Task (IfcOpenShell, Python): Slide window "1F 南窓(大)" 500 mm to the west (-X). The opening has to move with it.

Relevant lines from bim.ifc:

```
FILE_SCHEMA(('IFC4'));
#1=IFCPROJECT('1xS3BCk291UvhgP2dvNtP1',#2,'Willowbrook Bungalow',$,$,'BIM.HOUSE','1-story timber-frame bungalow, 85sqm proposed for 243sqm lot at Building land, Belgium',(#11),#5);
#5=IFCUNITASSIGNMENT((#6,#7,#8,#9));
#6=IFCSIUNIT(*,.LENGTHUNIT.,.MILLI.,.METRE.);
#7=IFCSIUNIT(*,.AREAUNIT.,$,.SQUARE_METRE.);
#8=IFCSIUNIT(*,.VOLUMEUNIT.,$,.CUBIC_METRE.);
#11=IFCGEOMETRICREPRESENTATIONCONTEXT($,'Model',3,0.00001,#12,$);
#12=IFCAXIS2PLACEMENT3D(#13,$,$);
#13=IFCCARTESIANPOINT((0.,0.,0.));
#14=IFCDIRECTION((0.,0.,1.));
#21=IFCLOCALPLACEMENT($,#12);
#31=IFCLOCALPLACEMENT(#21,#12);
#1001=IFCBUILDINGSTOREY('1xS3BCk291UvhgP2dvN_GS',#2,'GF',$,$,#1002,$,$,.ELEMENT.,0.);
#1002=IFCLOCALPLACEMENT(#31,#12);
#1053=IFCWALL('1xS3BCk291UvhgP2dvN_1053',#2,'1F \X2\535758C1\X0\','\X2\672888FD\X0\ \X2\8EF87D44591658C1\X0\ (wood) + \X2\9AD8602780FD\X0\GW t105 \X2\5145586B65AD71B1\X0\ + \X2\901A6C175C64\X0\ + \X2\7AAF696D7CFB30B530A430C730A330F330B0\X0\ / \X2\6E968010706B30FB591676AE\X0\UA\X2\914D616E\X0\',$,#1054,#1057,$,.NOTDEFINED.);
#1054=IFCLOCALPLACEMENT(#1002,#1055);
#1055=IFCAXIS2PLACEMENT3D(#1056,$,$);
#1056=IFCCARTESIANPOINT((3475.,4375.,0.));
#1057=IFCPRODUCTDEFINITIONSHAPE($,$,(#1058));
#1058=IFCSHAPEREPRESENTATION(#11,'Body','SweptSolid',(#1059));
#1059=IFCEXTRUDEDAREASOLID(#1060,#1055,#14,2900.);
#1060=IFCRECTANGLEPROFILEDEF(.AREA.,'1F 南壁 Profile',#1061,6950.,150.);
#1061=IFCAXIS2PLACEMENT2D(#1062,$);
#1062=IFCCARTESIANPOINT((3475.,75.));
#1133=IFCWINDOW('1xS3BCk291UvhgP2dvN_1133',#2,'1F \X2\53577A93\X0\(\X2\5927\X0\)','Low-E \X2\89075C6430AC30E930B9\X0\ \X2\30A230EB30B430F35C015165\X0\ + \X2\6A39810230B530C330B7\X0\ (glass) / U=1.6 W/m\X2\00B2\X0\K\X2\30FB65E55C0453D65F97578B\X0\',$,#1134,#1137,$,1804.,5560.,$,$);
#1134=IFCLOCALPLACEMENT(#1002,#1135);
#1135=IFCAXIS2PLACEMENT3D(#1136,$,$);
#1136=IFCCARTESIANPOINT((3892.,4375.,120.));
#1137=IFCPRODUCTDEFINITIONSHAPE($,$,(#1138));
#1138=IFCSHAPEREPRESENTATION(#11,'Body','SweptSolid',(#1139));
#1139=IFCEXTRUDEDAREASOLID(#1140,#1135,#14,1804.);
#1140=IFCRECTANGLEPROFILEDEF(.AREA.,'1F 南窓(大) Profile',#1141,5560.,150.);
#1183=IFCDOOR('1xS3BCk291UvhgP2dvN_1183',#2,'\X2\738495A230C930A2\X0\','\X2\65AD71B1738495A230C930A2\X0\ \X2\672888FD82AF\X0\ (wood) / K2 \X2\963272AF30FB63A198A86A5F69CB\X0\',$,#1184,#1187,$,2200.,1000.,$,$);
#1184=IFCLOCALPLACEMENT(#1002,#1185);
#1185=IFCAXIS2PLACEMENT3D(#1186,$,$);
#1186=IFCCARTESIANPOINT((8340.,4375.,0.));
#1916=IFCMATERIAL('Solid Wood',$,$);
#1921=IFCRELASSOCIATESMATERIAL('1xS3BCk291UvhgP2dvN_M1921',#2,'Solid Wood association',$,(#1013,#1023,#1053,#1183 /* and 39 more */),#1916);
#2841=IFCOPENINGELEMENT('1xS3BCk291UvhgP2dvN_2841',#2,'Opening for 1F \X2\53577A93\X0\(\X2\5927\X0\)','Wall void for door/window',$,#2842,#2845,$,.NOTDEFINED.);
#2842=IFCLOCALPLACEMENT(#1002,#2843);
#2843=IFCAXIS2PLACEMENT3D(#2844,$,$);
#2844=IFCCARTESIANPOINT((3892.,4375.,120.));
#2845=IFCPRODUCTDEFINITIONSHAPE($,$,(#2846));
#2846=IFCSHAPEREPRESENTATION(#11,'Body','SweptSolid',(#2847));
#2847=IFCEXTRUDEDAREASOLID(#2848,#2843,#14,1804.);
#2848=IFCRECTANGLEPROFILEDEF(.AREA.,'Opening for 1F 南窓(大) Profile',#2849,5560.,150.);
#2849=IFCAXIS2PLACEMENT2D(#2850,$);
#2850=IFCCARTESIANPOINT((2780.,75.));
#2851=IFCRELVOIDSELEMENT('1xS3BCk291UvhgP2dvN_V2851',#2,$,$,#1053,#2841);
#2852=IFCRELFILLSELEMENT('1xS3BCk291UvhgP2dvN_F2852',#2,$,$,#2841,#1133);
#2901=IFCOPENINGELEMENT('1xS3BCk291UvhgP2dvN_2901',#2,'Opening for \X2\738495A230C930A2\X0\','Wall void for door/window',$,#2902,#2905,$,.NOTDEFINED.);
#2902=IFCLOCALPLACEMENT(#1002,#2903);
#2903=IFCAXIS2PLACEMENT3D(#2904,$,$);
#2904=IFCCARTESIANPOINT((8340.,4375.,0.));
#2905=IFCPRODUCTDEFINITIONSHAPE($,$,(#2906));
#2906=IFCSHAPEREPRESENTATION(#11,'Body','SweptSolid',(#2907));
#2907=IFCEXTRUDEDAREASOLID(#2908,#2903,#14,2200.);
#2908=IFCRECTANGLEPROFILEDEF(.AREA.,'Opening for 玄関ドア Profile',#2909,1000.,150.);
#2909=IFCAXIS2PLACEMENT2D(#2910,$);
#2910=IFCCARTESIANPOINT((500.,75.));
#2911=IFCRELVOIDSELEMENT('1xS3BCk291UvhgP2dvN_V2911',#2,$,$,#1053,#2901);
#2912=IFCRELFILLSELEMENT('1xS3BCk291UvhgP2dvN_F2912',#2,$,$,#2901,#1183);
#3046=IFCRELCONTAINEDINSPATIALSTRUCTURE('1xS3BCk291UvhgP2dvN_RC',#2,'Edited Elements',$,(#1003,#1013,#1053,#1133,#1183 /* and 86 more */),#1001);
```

```python
import ifcopenshell
import ifcopenshell.api.geometry
import ifcopenshell.util.placement
import ifcopenshell.util.unit

model = ifcopenshell.open("bim.ifc")
unit_scale = ifcopenshell.util.unit.calculate_unit_scale(model)

window = model.by_id(1133)
opening = window.FillsVoids[0].RelatingOpeningElement
wall = opening.VoidsElements[0].RelatingBuildingElement

wall_matrix = ifcopenshell.util.placement.get_local_placement(wall.ObjectPlacement)
shift = wall_matrix[:3, 0] * -0.5 / unit_scale
before = ifcopenshell.util.placement.get_local_placement(window.ObjectPlacement)[:3, 3].copy()

# The window is not placed relative to its opening, so move both.
for product in (opening, window):
    matrix = ifcopenshell.util.placement.get_local_placement(product.ObjectPlacement)
    matrix[:3, 3] += shift
    ifcopenshell.api.geometry.edit_object_placement(model, product=product, matrix=matrix, is_si=False)

after = ifcopenshell.util.placement.get_local_placement(window.ObjectPlacement)[:3, 3]
print("window moved by", (after - before).round(3) + 0.0)

model.write("bim_updated.ifc")
```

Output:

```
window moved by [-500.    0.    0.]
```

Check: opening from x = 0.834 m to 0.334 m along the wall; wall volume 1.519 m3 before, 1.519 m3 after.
